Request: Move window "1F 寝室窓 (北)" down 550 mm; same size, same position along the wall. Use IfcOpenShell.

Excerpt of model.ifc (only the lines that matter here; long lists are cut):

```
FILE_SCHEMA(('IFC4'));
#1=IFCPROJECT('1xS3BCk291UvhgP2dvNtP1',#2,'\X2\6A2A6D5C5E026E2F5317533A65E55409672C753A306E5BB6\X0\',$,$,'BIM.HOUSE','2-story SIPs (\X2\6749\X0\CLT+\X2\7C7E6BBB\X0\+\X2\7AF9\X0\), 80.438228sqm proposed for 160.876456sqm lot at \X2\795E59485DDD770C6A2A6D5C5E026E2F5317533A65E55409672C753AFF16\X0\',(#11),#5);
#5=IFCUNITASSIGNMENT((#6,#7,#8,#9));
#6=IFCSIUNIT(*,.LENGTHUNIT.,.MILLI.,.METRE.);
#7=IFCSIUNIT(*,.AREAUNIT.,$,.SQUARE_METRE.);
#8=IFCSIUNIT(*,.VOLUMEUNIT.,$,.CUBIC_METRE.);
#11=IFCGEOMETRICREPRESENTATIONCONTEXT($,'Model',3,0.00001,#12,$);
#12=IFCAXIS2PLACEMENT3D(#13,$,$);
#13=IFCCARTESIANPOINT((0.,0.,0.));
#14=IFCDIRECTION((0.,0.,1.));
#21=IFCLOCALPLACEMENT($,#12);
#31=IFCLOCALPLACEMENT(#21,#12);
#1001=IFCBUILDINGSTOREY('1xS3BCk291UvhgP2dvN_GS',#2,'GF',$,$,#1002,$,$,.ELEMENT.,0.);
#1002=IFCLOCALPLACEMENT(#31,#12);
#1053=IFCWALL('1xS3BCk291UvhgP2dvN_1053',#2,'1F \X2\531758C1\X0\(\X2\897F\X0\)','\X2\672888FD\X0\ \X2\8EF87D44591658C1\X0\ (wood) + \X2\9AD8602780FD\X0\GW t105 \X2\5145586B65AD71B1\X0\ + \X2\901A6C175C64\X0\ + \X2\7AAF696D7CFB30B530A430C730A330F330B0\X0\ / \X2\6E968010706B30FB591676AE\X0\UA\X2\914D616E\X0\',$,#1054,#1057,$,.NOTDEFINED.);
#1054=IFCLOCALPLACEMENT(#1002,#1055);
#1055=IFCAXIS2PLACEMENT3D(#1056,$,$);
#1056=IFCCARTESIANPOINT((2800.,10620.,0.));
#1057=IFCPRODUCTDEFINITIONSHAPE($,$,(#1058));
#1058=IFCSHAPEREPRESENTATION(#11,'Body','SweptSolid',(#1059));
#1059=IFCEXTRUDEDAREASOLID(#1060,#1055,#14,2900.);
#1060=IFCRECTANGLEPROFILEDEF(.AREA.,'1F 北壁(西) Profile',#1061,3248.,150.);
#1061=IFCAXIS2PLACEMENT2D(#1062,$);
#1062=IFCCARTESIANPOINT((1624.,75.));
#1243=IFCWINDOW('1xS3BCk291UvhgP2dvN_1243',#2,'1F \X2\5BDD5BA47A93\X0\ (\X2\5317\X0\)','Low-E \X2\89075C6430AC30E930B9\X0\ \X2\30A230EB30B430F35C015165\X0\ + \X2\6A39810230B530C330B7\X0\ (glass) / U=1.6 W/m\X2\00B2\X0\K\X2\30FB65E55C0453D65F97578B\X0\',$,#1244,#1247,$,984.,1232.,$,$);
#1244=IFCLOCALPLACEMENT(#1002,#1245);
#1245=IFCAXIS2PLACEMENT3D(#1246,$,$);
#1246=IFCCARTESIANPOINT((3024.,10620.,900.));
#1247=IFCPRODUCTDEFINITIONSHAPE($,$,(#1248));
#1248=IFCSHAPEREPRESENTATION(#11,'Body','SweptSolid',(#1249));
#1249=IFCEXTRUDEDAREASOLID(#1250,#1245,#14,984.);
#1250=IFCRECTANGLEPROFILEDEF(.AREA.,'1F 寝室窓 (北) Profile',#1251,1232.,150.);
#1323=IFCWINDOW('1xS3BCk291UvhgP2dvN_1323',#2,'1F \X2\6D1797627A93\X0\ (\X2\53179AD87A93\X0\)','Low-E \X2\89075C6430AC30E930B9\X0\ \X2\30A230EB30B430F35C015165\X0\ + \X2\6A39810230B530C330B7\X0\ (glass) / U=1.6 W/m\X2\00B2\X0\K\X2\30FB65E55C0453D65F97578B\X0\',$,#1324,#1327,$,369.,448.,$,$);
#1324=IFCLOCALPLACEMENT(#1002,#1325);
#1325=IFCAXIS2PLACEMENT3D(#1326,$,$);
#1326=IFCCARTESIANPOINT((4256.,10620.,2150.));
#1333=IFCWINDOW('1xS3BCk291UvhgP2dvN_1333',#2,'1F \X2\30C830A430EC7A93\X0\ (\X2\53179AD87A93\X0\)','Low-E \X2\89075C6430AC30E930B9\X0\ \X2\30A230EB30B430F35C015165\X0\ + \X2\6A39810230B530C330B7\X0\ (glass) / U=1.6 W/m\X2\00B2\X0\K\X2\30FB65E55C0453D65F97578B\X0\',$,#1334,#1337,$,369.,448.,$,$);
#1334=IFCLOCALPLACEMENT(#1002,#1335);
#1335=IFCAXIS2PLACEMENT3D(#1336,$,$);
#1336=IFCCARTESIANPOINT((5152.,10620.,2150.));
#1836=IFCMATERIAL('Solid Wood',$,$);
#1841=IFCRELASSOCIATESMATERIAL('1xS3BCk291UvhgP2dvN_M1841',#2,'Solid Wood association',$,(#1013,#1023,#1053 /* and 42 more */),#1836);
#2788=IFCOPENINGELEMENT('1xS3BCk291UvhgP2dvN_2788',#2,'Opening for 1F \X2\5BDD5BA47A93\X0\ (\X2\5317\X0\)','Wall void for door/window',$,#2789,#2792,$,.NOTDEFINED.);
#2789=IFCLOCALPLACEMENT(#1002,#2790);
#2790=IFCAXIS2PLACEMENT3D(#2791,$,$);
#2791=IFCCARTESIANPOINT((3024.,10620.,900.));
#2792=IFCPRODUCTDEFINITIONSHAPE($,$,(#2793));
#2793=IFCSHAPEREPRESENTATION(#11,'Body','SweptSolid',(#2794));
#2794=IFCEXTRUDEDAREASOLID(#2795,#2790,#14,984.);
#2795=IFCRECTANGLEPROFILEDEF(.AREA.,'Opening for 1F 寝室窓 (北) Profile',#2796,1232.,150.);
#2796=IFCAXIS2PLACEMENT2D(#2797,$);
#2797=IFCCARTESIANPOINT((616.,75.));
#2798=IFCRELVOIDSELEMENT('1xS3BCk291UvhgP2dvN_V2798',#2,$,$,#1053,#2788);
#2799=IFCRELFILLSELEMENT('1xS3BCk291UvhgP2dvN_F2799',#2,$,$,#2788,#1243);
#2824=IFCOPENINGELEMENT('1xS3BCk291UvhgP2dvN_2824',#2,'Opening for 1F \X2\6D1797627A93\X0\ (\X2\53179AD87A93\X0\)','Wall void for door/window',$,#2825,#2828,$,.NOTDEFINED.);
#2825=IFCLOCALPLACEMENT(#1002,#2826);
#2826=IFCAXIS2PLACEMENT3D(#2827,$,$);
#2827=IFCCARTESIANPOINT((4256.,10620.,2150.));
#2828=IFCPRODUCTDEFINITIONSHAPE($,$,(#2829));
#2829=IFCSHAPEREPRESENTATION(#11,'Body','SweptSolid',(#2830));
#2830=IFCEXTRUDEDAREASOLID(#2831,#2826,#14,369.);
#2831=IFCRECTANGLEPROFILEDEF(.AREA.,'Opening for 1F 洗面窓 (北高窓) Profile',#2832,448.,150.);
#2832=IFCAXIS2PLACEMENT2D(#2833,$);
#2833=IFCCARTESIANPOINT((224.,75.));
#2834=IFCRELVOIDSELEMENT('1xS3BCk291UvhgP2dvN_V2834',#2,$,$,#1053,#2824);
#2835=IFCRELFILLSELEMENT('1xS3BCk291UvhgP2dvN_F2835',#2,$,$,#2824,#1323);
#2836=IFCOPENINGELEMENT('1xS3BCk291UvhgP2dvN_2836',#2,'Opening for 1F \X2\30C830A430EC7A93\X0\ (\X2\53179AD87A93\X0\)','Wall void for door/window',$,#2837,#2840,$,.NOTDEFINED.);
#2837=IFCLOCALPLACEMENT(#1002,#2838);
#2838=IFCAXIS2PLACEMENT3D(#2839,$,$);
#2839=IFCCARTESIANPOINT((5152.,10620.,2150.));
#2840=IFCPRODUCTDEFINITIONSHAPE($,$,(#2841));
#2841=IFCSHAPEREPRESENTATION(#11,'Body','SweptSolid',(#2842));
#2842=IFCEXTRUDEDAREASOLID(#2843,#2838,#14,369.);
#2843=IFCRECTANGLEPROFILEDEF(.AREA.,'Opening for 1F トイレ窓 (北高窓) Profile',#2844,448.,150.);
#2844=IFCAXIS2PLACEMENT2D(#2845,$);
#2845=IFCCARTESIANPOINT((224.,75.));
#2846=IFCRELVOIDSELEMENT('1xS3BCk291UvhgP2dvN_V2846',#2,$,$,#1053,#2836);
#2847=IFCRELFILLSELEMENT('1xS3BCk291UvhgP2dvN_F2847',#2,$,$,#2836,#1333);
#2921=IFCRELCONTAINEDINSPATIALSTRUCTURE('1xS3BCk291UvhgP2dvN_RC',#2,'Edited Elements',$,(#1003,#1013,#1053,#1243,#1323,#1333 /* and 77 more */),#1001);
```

```python
import numpy as np
import ifcopenshell
import ifcopenshell.api.geometry
import ifcopenshell.util.placement
import ifcopenshell.util.unit

model = ifcopenshell.open("model.ifc")
unit_scale = ifcopenshell.util.unit.calculate_unit_scale(model)

window = model.by_id(1243)
opening = window.FillsVoids[0].RelatingOpeningElement
dz = -0.55 / unit_scale

shift = np.array([0.0, 0.0, dz])
# The window is not placed relative to its opening, so move both.
for product in (opening, window):
    matrix = ifcopenshell.util.placement.get_local_placement(product.ObjectPlacement)
    matrix[:3, 3] += shift
    ifcopenshell.api.geometry.edit_object_placement(model, product=product, matrix=matrix, is_si=False)

print(f"moved by {dz * unit_scale:+.3f} m")

model.write("model_edited.ifc")
```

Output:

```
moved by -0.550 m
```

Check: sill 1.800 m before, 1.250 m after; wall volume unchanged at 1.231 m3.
